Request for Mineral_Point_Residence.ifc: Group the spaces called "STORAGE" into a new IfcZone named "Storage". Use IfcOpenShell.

First a look at what the model holds.

```python
import ifcopenshell

model = ifcopenshell.open("Mineral_Point_Residence.ifc")
print(model.schema)
seen = {}
for space in model.by_type("IfcSpace"):
    seen[space.LongName] = seen.get(space.LongName, 0) + 1
for name, count in sorted(seen.items(), key=str):
    print(count, "x", name)
print("zones:", [z.Name for z in model.by_type("IfcZone")][:20])
```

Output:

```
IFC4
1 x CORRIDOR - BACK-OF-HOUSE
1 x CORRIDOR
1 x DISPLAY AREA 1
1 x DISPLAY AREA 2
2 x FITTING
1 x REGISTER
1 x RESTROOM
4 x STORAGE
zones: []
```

```python
import ifcopenshell
import ifcopenshell.api.group
import ifcopenshell.api.root

model = ifcopenshell.open("Mineral_Point_Residence.ifc")

names = {"STORAGE"}
spaces = [s for s in model.by_type("IfcSpace") if s.LongName in names]

zone = ifcopenshell.api.root.create_entity(model, ifc_class="IfcZone", name="Storage")
ifcopenshell.api.group.assign_group(model, products=spaces, group=zone)
print(len(spaces), "spaces in", zone.Name)

model.write("Mineral_Point_Residence_v2.ifc")
```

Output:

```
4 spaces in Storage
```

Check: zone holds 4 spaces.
